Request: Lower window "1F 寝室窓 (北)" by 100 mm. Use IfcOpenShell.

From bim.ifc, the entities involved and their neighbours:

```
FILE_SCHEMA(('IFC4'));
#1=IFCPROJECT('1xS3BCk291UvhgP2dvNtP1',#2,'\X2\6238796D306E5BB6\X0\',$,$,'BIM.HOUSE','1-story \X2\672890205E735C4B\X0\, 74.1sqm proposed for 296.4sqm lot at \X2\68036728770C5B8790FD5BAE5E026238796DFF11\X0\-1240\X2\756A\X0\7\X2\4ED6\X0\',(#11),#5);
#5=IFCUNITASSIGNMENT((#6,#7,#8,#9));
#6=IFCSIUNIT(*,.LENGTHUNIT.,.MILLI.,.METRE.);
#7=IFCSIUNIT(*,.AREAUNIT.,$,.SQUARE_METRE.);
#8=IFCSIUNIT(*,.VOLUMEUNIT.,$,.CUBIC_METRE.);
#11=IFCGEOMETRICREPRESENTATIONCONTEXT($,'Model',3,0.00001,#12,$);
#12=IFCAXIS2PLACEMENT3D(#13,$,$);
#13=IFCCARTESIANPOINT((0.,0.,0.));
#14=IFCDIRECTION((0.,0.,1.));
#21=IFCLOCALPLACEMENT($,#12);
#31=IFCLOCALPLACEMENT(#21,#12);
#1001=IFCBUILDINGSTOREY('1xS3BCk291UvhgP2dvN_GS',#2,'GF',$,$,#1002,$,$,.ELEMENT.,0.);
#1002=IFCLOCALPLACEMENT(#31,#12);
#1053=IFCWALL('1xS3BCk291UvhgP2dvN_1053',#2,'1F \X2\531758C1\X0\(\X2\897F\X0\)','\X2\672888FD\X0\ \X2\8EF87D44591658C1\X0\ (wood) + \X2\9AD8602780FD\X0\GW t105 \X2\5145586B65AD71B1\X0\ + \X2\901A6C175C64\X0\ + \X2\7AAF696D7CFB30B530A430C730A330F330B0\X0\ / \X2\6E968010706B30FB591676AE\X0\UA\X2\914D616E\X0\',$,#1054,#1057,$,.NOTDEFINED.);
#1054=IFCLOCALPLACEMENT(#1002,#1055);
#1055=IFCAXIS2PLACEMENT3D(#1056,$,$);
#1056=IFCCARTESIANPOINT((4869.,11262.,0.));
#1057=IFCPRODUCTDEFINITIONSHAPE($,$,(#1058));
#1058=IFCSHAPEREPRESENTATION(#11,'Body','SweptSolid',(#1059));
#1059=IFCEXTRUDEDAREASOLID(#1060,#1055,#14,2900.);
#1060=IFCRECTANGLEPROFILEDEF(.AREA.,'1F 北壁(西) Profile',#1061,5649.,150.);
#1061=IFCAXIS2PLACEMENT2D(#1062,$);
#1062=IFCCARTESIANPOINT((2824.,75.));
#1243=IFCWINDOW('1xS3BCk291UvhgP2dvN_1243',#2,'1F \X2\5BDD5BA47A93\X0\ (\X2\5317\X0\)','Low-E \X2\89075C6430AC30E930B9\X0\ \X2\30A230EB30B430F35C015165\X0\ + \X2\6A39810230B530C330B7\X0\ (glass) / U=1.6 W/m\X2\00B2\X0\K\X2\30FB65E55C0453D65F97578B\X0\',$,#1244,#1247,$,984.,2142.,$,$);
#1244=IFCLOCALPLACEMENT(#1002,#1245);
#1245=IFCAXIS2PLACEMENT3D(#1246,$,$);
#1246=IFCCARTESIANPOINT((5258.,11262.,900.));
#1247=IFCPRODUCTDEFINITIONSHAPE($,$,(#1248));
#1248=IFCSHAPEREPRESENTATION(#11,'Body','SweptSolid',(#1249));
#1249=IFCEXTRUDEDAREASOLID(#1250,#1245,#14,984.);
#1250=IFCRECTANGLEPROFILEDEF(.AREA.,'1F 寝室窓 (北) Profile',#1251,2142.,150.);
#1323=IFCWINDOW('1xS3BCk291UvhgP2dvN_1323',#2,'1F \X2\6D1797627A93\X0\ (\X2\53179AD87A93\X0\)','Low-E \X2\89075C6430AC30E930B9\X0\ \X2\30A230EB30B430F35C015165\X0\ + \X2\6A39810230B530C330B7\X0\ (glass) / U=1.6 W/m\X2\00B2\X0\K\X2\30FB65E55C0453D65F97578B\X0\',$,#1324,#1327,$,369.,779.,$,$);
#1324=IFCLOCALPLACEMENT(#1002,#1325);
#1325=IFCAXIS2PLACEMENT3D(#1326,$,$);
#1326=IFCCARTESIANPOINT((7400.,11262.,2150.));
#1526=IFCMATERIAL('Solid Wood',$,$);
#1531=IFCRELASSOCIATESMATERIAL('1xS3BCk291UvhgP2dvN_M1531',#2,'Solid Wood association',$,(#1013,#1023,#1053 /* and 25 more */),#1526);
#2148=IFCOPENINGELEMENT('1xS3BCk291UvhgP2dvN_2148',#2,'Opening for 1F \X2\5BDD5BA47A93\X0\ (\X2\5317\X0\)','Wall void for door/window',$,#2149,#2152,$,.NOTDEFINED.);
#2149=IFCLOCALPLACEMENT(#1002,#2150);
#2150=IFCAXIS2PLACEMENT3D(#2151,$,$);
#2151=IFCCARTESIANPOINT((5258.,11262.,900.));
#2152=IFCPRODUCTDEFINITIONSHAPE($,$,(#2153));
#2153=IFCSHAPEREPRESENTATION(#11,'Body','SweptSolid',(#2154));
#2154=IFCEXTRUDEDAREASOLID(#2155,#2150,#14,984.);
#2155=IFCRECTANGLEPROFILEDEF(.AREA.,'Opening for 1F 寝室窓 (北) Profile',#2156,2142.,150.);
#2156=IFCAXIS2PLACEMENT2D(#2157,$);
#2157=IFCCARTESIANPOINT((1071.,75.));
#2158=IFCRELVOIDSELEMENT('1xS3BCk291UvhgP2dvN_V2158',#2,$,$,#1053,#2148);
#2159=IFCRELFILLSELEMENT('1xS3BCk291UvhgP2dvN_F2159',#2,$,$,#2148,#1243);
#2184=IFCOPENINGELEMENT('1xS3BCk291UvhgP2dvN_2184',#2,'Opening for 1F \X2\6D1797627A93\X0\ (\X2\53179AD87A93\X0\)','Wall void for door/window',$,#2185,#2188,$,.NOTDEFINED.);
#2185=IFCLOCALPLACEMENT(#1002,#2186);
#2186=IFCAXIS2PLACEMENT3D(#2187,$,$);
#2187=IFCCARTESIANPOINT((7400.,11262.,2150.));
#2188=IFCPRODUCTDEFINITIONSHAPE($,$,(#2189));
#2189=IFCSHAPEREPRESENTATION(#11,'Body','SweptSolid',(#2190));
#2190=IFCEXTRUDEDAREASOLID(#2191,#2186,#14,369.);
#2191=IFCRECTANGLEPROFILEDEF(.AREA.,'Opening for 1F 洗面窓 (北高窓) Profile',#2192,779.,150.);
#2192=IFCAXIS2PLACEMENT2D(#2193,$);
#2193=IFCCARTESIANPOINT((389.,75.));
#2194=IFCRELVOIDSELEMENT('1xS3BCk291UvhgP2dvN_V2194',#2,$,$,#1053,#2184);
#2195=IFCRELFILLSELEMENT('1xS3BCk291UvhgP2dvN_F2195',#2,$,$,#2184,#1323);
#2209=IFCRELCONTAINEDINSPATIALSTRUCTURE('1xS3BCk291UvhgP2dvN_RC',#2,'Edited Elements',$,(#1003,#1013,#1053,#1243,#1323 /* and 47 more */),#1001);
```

```python
import numpy as np
import ifcopenshell
import ifcopenshell.api.geometry
import ifcopenshell.util.placement
import ifcopenshell.util.unit

model = ifcopenshell.open("bim.ifc")
unit_scale = ifcopenshell.util.unit.calculate_unit_scale(model)

window = model.by_guid("1xS3BCk291UvhgP2dvN_1243")
opening = window.FillsVoids[0].RelatingOpeningElement
dz = -100.0

shift = np.array([0.0, 0.0, dz])
# The window is not placed relative to its opening, so move both.
for product in (opening, window):
    matrix = ifcopenshell.util.placement.get_local_placement(product.ObjectPlacement)
    matrix[:3, 3] += shift
    ifcopenshell.api.geometry.edit_object_placement(model, product=product, matrix=matrix, is_si=False)

print(f"moved by {dz * unit_scale:+.3f} m")

model.write("bim_rev.ifc")
```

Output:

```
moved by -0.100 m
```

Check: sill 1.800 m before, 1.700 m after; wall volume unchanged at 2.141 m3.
